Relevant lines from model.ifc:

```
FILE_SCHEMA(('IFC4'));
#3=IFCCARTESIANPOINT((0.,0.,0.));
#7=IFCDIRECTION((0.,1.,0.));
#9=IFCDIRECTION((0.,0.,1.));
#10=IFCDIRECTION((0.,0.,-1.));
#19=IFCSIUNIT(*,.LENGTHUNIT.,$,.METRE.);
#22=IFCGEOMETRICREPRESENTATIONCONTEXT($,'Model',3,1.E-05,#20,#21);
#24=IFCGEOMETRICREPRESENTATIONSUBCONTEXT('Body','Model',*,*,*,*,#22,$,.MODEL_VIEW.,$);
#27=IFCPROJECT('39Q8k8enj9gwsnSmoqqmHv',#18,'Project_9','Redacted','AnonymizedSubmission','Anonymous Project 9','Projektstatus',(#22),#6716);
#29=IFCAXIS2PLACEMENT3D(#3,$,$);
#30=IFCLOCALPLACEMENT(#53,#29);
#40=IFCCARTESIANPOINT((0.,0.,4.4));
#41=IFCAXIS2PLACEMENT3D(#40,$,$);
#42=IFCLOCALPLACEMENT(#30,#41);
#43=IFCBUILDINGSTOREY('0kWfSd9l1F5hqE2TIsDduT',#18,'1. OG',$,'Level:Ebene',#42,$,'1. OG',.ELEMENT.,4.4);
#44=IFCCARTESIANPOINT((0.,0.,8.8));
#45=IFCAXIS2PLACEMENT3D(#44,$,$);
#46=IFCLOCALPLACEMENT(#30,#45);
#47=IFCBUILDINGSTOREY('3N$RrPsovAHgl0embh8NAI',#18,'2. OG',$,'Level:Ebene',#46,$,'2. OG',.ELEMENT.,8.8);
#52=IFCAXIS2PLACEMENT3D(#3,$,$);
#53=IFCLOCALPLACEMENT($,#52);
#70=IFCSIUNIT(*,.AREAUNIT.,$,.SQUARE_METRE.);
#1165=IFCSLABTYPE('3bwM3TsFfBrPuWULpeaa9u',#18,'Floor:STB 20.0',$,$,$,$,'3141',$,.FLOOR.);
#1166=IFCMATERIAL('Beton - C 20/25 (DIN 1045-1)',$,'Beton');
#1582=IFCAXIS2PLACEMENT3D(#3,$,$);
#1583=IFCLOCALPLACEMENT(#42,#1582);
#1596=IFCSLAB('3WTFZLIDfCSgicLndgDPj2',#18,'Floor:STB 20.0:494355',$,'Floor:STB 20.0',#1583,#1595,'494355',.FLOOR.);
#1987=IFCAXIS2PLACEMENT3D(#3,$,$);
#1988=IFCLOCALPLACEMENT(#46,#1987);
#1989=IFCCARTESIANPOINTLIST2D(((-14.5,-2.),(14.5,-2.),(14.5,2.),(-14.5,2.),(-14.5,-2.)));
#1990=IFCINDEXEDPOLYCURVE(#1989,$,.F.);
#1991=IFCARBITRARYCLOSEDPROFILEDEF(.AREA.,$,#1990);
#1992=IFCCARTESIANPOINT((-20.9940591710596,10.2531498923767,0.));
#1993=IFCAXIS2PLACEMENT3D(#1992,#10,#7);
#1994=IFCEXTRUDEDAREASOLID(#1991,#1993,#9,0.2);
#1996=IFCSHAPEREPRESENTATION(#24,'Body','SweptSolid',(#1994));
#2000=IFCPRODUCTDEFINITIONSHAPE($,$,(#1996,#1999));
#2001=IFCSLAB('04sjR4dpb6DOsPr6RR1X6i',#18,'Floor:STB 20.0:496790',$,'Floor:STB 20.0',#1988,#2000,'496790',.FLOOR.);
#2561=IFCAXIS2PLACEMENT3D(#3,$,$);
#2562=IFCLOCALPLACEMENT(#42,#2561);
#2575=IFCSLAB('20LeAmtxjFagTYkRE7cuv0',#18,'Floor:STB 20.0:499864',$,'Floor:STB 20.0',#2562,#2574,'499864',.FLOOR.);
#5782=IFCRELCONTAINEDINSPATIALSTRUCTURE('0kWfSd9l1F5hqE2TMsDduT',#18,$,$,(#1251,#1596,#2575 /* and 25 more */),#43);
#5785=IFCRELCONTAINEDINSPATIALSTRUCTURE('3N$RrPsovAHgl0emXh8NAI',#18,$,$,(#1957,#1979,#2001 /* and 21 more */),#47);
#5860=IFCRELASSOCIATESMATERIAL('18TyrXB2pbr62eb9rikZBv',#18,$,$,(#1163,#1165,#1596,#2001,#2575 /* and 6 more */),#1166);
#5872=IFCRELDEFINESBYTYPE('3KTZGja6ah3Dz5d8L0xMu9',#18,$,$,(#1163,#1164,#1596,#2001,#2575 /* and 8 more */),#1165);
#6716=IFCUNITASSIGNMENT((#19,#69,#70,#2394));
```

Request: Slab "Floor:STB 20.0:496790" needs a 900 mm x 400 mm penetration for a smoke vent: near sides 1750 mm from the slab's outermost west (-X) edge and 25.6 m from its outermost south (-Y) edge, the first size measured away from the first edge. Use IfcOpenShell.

```python
import numpy as np
import ifcopenshell
import ifcopenshell.api.feature
import ifcopenshell.api.geometry
import ifcopenshell.api.root
import ifcopenshell.geom
import ifcopenshell.util.placement
import ifcopenshell.util.representation
import ifcopenshell.util.shape
import ifcopenshell.util.unit

model = ifcopenshell.open("model.ifc")
unit_scale = ifcopenshell.util.unit.calculate_unit_scale(model)
settings = ifcopenshell.geom.settings()


def volume(element):
    """Net volume in cubic metres, openings subtracted."""
    shape = ifcopenshell.geom.create_shape(settings, element)
    return ifcopenshell.util.shape.get_volume(shape.geometry)


slab = model.by_guid("04sjR4dpb6DOsPr6RR1X6i")
before = volume(slab)

# Extent in the slab's own axes, in metres. The edges named are its -X and -Y sides.
slab_shape = ifcopenshell.geom.create_shape(settings, slab)
vertices = ifcopenshell.util.shape.get_vertices(slab_shape.geometry)
x_min, y_min, bottom = vertices.min(axis=0)
top = vertices[:, 2].max()

opening = ifcopenshell.api.root.create_entity(model, ifc_class="IfcOpeningElement", name="Smoke vent opening", predefined_type="OPENING")
context = ifcopenshell.util.representation.get_context(model, "Model", "Body", "MODEL_VIEW")
width, depth = 0.9, 0.4
outline = [(0.0, 0.0), (width, 0.0), (width, depth), (0.0, depth), (0.0, 0.0)]
# Overshoot both faces by 50 mm so the cut is clean.
shape = ifcopenshell.api.geometry.add_slab_representation(
    model, context=context, depth=top - bottom + 0.1, polyline=outline
)
ifcopenshell.api.geometry.assign_representation(model, product=opening, representation=shape)

matrix = ifcopenshell.util.placement.get_local_placement(slab.ObjectPlacement)
matrix[:, 3] = matrix @ np.append(np.array([x_min + 1.75, y_min + 25.6, bottom - 0.05]) / unit_scale, 1.0)
ifcopenshell.api.geometry.edit_object_placement(model, product=opening, matrix=matrix, is_si=False)
ifcopenshell.api.feature.add_feature(model, feature=opening, element=slab)

after = volume(slab)

print(f"slab volume {before:.3f} -> {after:.3f} m3")

model.write("model_v2.ifc")
```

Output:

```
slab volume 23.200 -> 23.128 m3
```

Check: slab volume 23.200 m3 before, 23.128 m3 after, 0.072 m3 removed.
